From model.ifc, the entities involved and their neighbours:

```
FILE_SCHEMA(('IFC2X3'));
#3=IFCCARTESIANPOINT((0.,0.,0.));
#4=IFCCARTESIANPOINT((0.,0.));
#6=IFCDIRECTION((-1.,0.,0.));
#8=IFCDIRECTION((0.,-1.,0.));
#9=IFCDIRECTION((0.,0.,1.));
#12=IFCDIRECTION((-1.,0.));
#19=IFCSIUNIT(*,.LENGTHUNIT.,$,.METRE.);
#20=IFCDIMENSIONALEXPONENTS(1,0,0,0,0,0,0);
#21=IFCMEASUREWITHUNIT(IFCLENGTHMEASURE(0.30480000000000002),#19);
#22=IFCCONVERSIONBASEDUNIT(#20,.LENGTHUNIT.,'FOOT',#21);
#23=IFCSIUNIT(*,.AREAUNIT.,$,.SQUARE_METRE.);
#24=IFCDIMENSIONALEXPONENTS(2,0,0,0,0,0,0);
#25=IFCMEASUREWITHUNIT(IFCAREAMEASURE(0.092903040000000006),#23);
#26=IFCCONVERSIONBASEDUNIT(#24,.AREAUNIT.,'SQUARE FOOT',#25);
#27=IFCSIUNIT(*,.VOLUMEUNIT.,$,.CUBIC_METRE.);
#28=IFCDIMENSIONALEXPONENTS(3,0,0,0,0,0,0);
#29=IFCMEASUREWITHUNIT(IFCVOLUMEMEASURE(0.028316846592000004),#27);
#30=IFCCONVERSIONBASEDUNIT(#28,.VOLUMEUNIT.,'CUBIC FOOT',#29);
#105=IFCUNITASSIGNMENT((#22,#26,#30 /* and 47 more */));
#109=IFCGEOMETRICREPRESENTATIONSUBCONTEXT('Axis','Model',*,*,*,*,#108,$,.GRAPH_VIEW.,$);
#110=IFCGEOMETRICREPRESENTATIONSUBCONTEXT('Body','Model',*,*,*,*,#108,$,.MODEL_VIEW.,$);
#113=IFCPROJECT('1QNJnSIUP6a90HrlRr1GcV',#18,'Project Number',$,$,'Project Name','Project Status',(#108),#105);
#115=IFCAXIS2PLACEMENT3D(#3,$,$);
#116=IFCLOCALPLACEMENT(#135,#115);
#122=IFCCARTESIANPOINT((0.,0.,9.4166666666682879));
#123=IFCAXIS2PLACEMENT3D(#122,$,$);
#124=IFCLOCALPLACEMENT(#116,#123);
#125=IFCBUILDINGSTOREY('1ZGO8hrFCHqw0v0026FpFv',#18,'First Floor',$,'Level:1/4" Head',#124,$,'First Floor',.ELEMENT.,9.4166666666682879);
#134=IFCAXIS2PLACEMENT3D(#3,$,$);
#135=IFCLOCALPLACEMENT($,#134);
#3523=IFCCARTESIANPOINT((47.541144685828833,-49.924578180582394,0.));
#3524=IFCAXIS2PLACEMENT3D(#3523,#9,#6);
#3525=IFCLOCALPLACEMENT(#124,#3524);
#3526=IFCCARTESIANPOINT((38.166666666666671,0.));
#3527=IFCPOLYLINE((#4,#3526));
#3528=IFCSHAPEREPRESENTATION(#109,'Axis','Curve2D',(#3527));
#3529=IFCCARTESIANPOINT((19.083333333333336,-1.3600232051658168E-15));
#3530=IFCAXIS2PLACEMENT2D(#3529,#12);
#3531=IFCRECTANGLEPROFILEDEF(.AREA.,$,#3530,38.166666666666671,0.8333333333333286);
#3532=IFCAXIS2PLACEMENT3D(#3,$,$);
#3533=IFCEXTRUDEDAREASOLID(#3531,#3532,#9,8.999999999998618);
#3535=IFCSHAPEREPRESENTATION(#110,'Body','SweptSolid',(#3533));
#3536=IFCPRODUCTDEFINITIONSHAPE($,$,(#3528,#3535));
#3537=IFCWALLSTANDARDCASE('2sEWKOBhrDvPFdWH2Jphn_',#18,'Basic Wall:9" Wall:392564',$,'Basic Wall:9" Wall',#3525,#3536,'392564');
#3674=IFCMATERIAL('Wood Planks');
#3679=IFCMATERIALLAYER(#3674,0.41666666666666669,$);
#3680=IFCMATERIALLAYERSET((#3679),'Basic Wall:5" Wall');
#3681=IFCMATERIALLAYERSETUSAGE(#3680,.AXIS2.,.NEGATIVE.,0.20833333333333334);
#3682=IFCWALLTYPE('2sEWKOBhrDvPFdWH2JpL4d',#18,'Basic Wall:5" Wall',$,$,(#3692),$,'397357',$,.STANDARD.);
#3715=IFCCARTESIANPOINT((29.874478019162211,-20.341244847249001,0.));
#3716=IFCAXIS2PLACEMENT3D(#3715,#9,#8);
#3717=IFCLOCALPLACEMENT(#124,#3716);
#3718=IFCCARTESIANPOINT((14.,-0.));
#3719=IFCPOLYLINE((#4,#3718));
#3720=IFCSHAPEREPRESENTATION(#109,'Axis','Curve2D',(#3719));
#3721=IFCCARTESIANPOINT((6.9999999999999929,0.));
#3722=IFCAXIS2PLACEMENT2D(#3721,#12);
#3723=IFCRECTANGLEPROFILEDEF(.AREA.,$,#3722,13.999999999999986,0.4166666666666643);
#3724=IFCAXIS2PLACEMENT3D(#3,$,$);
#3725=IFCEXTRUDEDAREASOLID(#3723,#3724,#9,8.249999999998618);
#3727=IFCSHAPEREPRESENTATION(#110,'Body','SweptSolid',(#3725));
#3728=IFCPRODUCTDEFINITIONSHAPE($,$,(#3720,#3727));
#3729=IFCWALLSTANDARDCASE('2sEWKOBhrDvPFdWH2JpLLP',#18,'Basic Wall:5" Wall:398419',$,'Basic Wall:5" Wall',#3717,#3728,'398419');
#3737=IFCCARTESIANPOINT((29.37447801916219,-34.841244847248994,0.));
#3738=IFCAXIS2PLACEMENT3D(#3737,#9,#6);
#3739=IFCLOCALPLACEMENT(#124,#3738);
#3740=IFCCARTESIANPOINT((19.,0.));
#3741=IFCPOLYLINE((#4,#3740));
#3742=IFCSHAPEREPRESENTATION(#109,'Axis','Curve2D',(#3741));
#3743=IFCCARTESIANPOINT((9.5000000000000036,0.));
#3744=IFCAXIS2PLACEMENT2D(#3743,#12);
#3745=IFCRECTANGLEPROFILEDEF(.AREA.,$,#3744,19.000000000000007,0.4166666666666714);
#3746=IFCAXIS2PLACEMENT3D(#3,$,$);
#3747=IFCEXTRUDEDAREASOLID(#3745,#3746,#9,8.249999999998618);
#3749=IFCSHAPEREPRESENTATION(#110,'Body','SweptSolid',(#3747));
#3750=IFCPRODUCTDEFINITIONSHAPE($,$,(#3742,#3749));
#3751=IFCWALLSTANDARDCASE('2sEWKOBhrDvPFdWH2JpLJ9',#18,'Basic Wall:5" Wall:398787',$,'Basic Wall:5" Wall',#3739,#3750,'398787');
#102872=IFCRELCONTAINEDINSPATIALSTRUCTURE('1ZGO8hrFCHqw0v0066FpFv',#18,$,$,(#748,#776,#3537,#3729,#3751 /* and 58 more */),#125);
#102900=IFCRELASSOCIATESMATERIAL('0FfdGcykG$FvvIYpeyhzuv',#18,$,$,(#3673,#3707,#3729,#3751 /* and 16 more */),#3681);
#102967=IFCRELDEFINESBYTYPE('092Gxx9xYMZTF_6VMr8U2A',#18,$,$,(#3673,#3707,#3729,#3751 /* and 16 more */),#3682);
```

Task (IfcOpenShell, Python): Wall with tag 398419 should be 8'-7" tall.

```python
import ifcopenshell
import ifcopenshell.geom
import ifcopenshell.util.representation
import ifcopenshell.util.shape
import ifcopenshell.util.unit

model = ifcopenshell.open("model.ifc")
unit_scale = ifcopenshell.util.unit.calculate_unit_scale(model)
settings = ifcopenshell.geom.settings()


def volume(element):
    """Net volume in cubic metres, openings subtracted."""
    shape = ifcopenshell.geom.create_shape(settings, element)
    return ifcopenshell.util.shape.get_volume(shape.geometry)


wall = model.by_guid("2sEWKOBhrDvPFdWH2JpLLP")
before = volume(wall)

body = ifcopenshell.util.representation.get_representation(wall, "Model", "Body")
solid = body.Items[0]
old_height = solid.Depth
solid.Depth = 103 * 0.0254 / unit_scale
after = volume(wall)

print(f"height {old_height:g} -> {solid.Depth:g}, volume {before:.3f} -> {after:.3f} m3")

model.write("model-out.ifc")
```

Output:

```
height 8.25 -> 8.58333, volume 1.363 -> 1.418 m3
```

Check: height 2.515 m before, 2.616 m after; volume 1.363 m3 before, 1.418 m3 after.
